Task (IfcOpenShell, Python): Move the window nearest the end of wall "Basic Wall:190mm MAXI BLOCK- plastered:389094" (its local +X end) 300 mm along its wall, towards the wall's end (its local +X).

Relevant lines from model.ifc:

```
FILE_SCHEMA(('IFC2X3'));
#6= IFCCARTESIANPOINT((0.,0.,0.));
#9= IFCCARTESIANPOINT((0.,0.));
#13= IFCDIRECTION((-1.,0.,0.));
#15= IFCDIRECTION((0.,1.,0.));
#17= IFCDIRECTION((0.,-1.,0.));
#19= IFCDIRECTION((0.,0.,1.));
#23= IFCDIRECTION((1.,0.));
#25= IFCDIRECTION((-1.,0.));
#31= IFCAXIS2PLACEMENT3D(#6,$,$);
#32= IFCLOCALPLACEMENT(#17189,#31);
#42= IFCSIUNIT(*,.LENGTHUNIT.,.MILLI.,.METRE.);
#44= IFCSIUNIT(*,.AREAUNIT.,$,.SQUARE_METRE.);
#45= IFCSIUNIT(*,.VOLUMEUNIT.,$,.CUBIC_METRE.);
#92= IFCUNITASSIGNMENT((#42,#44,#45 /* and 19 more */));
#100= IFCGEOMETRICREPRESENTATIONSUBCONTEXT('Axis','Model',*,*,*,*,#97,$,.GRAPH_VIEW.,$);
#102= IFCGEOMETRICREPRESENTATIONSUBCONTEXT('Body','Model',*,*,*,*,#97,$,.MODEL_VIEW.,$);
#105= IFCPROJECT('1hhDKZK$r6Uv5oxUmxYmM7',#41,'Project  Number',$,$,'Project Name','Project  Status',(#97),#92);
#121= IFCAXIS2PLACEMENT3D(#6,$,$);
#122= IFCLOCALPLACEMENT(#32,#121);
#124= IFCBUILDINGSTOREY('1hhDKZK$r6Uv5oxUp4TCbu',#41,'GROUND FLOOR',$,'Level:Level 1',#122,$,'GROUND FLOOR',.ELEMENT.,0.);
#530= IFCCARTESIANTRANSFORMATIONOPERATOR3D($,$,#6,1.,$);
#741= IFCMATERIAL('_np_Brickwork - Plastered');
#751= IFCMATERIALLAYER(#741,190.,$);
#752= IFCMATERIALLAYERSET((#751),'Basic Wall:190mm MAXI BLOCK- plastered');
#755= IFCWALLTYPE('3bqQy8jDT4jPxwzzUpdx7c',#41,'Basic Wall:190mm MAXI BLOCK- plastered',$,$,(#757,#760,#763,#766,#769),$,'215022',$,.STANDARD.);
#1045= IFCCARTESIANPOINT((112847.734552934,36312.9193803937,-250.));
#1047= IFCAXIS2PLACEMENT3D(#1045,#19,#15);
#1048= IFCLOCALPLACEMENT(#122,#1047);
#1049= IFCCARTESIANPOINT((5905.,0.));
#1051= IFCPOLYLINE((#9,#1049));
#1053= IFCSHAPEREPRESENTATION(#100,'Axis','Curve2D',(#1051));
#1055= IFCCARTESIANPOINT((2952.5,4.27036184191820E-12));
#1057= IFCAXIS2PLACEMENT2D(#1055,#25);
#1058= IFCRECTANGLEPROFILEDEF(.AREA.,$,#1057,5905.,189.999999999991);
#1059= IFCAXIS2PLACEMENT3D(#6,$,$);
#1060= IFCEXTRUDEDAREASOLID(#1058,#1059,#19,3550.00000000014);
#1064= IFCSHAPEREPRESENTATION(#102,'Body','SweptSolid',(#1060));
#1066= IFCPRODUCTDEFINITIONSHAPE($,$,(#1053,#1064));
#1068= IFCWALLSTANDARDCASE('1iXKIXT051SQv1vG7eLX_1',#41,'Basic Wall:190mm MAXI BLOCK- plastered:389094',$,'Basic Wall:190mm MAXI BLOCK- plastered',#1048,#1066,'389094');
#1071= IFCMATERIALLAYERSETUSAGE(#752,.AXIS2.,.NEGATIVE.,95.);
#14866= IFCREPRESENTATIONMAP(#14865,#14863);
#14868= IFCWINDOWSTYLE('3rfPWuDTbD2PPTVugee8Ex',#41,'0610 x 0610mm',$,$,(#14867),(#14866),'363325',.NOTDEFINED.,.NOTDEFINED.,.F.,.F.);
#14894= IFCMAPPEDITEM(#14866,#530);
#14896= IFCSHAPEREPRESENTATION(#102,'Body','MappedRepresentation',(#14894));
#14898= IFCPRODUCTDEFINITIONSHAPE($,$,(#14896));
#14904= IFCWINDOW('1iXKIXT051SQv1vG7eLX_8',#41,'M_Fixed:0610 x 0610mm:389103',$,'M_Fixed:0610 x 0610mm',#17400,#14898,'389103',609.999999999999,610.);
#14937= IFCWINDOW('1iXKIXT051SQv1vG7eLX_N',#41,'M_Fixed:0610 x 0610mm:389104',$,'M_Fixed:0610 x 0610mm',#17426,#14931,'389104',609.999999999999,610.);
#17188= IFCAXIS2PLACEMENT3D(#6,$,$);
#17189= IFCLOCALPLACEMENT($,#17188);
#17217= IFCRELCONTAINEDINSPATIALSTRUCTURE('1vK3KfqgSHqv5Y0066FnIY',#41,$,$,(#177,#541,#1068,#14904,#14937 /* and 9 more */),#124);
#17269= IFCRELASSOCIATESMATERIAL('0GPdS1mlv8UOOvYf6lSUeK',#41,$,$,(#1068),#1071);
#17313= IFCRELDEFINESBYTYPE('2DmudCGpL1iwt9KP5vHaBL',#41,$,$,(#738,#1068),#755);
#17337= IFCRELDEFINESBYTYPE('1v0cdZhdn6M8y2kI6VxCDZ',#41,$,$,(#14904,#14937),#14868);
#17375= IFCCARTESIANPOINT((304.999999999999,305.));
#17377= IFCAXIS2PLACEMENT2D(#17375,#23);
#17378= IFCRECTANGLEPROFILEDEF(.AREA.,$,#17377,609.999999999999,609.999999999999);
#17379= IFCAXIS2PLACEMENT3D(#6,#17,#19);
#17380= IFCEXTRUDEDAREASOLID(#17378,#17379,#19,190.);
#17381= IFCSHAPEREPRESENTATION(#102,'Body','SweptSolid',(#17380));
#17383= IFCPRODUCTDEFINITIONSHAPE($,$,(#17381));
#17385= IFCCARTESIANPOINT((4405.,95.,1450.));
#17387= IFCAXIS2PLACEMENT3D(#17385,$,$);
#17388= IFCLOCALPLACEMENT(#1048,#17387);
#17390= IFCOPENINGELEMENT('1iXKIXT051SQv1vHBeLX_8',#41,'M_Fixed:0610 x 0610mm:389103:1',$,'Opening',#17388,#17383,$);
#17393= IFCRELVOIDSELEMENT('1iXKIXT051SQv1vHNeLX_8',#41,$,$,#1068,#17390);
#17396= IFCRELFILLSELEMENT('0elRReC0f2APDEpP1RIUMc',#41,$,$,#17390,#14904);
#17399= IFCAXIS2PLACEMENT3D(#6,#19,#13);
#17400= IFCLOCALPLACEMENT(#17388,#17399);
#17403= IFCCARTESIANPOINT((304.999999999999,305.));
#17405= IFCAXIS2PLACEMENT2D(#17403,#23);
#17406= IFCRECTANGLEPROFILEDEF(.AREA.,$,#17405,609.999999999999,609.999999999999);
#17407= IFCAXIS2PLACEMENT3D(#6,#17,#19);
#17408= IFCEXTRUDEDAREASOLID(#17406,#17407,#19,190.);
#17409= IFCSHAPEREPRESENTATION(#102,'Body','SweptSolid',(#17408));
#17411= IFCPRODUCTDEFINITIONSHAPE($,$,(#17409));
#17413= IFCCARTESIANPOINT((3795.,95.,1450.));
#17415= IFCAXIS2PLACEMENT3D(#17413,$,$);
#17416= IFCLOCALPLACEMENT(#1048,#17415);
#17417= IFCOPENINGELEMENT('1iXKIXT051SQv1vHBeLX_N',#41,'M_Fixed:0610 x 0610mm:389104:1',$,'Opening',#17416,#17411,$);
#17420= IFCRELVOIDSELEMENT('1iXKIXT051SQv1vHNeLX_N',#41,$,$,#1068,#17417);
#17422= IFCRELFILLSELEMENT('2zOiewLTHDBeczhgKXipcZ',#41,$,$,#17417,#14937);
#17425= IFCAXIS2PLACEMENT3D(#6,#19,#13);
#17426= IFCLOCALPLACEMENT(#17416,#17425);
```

```python
import ifcopenshell
import ifcopenshell.api.geometry
import ifcopenshell.util.placement
import ifcopenshell.util.unit

model = ifcopenshell.open("model.ifc")
unit_scale = ifcopenshell.util.unit.calculate_unit_scale(model)

window = model.by_guid("1iXKIXT051SQv1vG7eLX_8")
opening = window.FillsVoids[0].RelatingOpeningElement
wall = opening.VoidsElements[0].RelatingBuildingElement

wall_matrix = ifcopenshell.util.placement.get_local_placement(wall.ObjectPlacement)
shift = wall_matrix[:3, 0] * 0.3 / unit_scale
before = ifcopenshell.util.placement.get_local_placement(window.ObjectPlacement)[:3, 3].copy()

# The window is placed relative to its opening, so it follows when the opening moves.
matrix = ifcopenshell.util.placement.get_local_placement(opening.ObjectPlacement)
matrix[:3, 3] += shift
ifcopenshell.api.geometry.edit_object_placement(
    model, product=opening, matrix=matrix, is_si=False, should_transform_children=True
)

after = ifcopenshell.util.placement.get_local_placement(window.ObjectPlacement)[:3, 3]
print("window moved by", (after - before).round(3) + 0.0)

model.write("model_edited.ifc")
```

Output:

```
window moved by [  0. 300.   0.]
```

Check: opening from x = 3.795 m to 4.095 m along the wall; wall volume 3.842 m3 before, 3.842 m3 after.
